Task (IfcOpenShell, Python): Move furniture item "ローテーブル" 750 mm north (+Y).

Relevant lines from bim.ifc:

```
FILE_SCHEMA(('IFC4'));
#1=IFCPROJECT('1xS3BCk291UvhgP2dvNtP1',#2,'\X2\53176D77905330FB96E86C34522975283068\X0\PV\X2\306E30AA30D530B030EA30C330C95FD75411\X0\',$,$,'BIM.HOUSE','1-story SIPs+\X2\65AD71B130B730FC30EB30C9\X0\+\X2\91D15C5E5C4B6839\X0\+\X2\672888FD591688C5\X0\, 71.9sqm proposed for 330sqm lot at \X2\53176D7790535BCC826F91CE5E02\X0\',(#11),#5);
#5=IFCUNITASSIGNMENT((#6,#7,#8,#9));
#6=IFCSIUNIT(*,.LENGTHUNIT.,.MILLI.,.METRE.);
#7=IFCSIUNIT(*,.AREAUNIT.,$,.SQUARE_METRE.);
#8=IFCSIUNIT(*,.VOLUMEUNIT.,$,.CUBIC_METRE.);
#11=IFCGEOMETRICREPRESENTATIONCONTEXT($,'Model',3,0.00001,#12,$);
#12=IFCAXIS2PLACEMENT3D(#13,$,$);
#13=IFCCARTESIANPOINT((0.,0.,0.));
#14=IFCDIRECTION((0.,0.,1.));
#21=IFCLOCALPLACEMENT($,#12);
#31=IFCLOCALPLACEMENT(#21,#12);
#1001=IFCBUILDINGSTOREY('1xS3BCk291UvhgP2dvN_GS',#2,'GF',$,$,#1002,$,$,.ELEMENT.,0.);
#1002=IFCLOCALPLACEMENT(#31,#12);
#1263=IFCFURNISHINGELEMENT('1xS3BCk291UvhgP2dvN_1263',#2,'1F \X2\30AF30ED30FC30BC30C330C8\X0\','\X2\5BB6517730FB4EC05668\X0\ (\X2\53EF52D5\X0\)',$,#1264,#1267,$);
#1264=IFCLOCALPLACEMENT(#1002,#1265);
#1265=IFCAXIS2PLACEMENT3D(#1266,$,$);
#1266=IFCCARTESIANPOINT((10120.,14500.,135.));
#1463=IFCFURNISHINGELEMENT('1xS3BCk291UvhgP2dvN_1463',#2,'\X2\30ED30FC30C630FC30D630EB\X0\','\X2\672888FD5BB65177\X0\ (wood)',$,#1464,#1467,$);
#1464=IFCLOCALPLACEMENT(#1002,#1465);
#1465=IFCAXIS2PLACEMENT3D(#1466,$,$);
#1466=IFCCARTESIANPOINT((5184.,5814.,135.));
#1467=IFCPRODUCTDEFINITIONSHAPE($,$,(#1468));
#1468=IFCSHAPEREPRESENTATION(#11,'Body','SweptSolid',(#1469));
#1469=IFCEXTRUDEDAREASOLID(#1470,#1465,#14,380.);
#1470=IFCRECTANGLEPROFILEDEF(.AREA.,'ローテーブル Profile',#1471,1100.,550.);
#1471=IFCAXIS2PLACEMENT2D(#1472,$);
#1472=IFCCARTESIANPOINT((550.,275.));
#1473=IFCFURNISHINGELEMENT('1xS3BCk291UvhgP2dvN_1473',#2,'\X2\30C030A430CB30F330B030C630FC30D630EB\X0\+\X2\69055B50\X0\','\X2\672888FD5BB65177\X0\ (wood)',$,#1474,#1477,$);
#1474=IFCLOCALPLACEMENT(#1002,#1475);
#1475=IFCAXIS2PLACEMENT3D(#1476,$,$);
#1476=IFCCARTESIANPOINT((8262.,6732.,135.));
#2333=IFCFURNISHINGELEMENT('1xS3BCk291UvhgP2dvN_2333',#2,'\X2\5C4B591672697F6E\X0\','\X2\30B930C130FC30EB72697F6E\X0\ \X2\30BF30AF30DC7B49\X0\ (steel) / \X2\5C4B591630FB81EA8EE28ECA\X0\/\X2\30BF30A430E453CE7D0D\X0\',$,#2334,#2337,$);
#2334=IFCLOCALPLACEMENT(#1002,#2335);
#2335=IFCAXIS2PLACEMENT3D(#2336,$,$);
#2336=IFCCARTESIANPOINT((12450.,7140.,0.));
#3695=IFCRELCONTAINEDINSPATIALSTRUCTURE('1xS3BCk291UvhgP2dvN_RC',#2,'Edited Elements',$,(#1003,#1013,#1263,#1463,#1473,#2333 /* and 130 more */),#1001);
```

```python
import ifcopenshell
import ifcopenshell.api.geometry
import ifcopenshell.util.placement
import ifcopenshell.util.unit

model = ifcopenshell.open("bim.ifc")
unit_scale = ifcopenshell.util.unit.calculate_unit_scale(model)

item = model.by_guid("1xS3BCk291UvhgP2dvN_1463")
matrix = ifcopenshell.util.placement.get_local_placement(item.ObjectPlacement)
matrix[1, 3] += 0.75 / unit_scale
ifcopenshell.api.geometry.edit_object_placement(model, product=item, matrix=matrix, is_si=False)

print(ifcopenshell.util.placement.get_local_placement(item.ObjectPlacement).round(3) + 0.0)

model.write("bim-out.ifc")
```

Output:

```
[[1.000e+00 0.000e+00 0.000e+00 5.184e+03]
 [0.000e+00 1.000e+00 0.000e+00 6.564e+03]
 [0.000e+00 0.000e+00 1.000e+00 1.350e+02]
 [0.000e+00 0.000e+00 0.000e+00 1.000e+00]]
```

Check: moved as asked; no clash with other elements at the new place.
